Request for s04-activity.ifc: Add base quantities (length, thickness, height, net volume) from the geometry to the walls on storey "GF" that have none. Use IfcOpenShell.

First a look at what the model holds.

```python
import ifcopenshell
import ifcopenshell.util.element
import ifcopenshell.util.unit

model = ifcopenshell.open("s04-activity.ifc")
print(model.schema)
for unit_type in ("LENGTHUNIT", "AREAUNIT", "VOLUMEUNIT"):
    print(unit_type, ifcopenshell.util.unit.calculate_unit_scale(model, unit_type))
storey = next(s for s in model.by_type("IfcBuildingStorey") if s.Name == "GF")
walls = [e for e in ifcopenshell.util.element.get_decomposition(storey) if e.is_a("IfcWall")]
for e in sorted(walls, key=lambda e: e.id()):
    print(e.id(), e.is_a(), e.Name, list(ifcopenshell.util.element.get_psets(e, qtos_only=True)), sep=" | ")
```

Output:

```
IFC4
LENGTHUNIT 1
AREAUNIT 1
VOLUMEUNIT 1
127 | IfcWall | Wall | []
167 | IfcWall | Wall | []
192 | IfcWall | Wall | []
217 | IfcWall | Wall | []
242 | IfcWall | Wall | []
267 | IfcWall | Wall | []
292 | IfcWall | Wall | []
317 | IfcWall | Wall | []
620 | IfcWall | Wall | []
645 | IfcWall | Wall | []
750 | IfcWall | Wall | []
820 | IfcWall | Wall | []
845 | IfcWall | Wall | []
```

```python
import ifcopenshell
import ifcopenshell.api.pset
import ifcopenshell.geom
import ifcopenshell.util.element
import ifcopenshell.util.shape
import ifcopenshell.util.unit

model = ifcopenshell.open("s04-activity.ifc")
unit_scale = ifcopenshell.util.unit.calculate_unit_scale(model)
volume_scale = ifcopenshell.util.unit.calculate_unit_scale(model, "VOLUMEUNIT")
settings = ifcopenshell.geom.settings()

storey = next(s for s in model.by_type("IfcBuildingStorey") if s.Name == "GF")
walls = [e for e in ifcopenshell.util.element.get_decomposition(storey) if e.is_a("IfcWall")]

for e in sorted(walls, key=lambda e: e.id()):
    if ifcopenshell.util.element.get_psets(e, qtos_only=True, should_inherit=False):
        continue
    # Geometry comes back in metres, in the element's own axes.
    shape = ifcopenshell.geom.create_shape(settings, e)
    values = {
        "Length": ifcopenshell.util.shape.get_x(shape.geometry) / unit_scale,
        "Width": ifcopenshell.util.shape.get_y(shape.geometry) / unit_scale,
        "Height": ifcopenshell.util.shape.get_z(shape.geometry) / unit_scale,
        "NetVolume": ifcopenshell.util.shape.get_volume(shape.geometry) / volume_scale,
    }
    qto = ifcopenshell.api.pset.add_qto(model, product=e, name="Qto_WallBaseQuantities")
    ifcopenshell.api.pset.edit_qto(model, qto=qto, properties=values)
    print(e.id(), {k: round(v, 3) for k, v in values.items()})

model.write("s04-activity_updated.ifc")
```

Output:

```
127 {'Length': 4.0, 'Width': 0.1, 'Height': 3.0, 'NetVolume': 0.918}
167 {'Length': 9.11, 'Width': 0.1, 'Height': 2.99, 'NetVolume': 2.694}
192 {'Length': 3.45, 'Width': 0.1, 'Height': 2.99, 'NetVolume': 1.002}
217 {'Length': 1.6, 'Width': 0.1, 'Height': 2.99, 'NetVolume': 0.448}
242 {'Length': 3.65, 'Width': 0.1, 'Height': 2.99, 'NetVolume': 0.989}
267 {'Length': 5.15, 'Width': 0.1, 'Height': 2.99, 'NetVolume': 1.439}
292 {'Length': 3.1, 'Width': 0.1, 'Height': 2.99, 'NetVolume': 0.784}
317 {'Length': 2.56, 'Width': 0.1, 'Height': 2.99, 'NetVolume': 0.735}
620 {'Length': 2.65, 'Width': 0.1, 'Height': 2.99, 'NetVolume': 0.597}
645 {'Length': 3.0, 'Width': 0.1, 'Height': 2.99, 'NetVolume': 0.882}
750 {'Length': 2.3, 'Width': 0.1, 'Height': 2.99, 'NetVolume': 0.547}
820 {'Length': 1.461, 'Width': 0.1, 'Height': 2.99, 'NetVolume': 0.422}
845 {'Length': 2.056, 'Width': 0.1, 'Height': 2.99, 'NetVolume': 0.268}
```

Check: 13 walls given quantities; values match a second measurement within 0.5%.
